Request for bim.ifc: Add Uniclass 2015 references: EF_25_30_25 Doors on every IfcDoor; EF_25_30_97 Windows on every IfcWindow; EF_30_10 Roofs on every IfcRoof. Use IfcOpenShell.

First a look at what the model holds.

```python
import ifcopenshell

model = ifcopenshell.open("bim.ifc")
print(model.schema)
print("classifications:", [c.Name for c in model.by_type("IfcClassification")])
for ifc_class in ("IfcDoor", "IfcRoof", "IfcStair", "IfcWall", "IfcWindow"):
    print(ifc_class, len(model.by_type(ifc_class)))
```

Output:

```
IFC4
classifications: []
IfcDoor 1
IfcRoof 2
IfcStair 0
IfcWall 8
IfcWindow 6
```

```python
import ifcopenshell
import ifcopenshell.api.classification

model = ifcopenshell.open("bim.ifc")

system = ifcopenshell.api.classification.add_classification(model, classification="Uniclass 2015")

codes = {
    "IfcDoor": ("EF_25_30_25", "Doors"),
    "IfcWindow": ("EF_25_30_97", "Windows"),
    "IfcRoof": ("EF_30_10", "Roofs"),
}
for ifc_class, (code, name) in codes.items():
    products = model.by_type(ifc_class)
    ifcopenshell.api.classification.add_reference(
        model, products=products, classification=system, identification=code, name=name
    )
    print(code, len(products))

model.write("bim_edited.ifc")
```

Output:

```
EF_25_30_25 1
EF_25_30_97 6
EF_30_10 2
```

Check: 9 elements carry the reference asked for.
